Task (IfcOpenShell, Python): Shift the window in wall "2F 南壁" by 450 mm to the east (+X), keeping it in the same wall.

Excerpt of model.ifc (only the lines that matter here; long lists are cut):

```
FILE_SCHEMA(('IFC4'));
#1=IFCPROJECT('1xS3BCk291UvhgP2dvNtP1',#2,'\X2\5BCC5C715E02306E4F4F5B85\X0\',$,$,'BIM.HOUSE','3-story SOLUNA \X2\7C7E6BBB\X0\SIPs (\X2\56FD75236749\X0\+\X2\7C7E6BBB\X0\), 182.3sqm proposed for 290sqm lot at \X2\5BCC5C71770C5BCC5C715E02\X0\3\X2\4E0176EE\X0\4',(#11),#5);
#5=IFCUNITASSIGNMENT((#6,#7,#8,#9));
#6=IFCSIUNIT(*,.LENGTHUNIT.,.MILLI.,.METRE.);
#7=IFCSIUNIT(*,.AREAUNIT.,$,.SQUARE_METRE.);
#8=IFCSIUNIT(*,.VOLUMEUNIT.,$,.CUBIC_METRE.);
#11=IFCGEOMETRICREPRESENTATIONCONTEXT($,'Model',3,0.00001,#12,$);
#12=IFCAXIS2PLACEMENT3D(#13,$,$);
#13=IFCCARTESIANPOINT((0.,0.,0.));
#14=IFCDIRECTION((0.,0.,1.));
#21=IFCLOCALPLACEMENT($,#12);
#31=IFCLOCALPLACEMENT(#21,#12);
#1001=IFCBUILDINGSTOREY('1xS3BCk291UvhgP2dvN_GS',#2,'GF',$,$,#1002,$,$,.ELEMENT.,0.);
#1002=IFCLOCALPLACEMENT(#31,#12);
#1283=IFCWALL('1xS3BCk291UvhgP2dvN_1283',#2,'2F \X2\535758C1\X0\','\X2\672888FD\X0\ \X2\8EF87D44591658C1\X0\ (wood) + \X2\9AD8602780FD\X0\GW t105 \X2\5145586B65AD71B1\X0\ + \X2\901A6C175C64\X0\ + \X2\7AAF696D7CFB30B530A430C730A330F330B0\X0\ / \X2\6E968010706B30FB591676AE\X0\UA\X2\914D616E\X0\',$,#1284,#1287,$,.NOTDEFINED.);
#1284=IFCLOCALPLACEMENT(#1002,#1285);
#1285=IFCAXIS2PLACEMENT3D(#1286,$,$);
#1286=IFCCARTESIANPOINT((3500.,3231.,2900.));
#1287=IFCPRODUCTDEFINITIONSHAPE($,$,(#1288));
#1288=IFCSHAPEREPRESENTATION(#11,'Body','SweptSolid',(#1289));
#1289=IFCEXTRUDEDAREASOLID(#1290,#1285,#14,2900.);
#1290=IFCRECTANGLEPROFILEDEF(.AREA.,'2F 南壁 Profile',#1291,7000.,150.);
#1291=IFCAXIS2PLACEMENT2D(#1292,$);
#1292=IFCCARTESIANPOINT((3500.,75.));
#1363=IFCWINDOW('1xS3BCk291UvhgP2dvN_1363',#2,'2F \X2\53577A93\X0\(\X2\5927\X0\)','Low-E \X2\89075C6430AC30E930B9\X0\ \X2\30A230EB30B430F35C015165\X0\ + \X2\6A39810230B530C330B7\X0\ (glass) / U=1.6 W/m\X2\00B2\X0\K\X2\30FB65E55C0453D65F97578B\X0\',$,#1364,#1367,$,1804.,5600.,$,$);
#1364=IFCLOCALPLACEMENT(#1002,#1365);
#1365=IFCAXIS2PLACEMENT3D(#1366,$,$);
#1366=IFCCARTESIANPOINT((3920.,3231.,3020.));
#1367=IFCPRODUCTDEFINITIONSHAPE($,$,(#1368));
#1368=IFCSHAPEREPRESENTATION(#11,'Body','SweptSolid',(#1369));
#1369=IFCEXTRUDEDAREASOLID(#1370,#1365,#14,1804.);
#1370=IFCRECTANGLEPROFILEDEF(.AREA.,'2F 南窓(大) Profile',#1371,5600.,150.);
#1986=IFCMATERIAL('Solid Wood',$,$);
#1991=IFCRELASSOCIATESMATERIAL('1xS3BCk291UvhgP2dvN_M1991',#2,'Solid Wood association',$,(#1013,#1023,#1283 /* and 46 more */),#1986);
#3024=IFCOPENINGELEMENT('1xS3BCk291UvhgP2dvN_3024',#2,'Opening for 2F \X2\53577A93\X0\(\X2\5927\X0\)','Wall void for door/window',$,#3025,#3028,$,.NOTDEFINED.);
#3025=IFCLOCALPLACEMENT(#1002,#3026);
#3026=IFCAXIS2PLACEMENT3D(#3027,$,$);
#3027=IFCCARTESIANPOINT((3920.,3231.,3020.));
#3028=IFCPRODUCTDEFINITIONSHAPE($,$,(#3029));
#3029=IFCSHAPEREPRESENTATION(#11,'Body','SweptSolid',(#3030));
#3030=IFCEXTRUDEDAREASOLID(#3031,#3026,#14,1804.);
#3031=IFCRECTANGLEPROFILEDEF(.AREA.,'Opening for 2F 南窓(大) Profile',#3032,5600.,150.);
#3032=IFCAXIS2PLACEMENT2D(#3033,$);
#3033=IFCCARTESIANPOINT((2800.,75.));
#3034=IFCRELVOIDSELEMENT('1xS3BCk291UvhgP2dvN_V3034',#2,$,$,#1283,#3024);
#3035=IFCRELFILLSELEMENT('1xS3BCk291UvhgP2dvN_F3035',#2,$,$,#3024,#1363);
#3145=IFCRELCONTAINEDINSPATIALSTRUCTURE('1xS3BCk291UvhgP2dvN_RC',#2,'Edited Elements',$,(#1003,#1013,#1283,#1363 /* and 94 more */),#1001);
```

```python
import ifcopenshell
import ifcopenshell.api.geometry
import ifcopenshell.util.placement

model = ifcopenshell.open("model.ifc")

window = model.by_guid("1xS3BCk291UvhgP2dvN_1363")
opening = window.FillsVoids[0].RelatingOpeningElement
wall = opening.VoidsElements[0].RelatingBuildingElement

wall_matrix = ifcopenshell.util.placement.get_local_placement(wall.ObjectPlacement)
shift = wall_matrix[:3, 0] * 450.0
before = ifcopenshell.util.placement.get_local_placement(window.ObjectPlacement)[:3, 3].copy()

# The window is not placed relative to its opening, so move both.
for product in (opening, window):
    matrix = ifcopenshell.util.placement.get_local_placement(product.ObjectPlacement)
    matrix[:3, 3] += shift
    ifcopenshell.api.geometry.edit_object_placement(model, product=product, matrix=matrix, is_si=False)

after = ifcopenshell.util.placement.get_local_placement(window.ObjectPlacement)[:3, 3]
print("window moved by", (after - before).round(3) + 0.0)

model.write("model_rev.ifc")
```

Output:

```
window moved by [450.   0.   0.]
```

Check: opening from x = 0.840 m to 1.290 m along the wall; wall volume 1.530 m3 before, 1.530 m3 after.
